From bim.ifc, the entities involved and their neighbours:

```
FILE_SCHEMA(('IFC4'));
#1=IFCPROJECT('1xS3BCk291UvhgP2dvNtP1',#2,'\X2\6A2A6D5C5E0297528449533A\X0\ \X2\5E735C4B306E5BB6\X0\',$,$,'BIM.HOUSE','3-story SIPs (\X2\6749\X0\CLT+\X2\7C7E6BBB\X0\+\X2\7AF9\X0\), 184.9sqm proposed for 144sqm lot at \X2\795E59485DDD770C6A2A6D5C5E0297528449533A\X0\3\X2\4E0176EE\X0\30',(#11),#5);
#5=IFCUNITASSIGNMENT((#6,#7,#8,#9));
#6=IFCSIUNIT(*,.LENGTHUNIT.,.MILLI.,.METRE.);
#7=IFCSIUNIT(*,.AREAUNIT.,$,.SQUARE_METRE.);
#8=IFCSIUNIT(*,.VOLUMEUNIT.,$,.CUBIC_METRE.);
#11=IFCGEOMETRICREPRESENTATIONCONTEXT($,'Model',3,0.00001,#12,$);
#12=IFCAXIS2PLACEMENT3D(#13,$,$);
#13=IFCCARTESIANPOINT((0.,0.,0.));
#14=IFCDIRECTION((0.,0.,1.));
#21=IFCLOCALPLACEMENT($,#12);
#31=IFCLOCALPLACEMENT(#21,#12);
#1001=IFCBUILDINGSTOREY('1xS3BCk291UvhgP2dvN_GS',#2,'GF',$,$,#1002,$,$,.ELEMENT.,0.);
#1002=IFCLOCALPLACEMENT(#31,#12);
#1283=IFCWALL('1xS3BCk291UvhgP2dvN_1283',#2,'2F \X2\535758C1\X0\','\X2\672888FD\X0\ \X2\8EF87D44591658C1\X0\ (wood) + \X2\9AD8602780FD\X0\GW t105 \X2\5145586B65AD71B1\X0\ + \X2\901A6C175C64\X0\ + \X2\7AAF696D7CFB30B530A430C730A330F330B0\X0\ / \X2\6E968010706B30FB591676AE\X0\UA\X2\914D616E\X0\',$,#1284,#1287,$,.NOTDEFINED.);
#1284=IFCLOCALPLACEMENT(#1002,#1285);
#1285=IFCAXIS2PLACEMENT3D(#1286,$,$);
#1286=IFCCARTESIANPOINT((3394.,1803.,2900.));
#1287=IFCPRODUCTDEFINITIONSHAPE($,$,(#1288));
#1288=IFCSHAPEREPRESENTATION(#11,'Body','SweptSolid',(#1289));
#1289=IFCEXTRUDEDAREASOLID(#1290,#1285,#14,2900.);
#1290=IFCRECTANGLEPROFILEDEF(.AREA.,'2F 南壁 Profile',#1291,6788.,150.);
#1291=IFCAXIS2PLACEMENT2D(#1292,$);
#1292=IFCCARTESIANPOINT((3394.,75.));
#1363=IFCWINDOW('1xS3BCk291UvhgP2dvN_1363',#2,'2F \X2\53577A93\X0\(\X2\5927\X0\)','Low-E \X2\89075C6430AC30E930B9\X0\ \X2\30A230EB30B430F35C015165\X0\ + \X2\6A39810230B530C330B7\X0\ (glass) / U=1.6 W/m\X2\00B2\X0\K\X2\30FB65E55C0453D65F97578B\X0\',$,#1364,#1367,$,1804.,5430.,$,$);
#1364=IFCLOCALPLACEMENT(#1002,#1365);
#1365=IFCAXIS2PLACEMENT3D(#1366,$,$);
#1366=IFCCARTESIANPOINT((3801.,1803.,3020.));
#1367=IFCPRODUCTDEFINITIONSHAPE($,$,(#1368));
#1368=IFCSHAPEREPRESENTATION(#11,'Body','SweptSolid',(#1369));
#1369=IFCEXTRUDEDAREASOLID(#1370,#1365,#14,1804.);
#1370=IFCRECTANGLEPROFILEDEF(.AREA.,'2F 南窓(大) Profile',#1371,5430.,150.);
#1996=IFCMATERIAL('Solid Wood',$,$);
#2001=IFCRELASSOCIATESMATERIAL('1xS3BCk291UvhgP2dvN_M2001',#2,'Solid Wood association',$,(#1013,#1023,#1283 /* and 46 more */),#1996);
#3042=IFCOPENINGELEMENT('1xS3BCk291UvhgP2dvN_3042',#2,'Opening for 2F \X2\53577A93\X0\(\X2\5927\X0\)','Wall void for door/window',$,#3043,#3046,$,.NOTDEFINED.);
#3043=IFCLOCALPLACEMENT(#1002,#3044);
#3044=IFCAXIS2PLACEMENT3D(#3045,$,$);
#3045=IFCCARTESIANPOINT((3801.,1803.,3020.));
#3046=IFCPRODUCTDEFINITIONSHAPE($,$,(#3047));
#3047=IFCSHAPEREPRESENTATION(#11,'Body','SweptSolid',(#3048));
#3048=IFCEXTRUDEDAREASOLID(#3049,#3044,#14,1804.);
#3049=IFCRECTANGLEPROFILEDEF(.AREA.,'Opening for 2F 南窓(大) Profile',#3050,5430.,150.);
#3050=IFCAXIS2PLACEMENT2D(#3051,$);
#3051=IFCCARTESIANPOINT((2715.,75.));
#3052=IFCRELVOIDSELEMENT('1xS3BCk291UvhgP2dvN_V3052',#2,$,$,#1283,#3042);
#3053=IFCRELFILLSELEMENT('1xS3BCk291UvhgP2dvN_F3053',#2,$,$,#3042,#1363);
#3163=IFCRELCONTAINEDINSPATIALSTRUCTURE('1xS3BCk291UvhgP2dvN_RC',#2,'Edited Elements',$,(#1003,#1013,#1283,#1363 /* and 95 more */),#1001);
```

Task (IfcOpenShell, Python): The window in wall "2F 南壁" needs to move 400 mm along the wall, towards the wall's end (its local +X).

```python
import ifcopenshell
import ifcopenshell.api.geometry
import ifcopenshell.util.placement
import ifcopenshell.util.unit

model = ifcopenshell.open("bim.ifc")
unit_scale = ifcopenshell.util.unit.calculate_unit_scale(model)

window = model.by_guid("1xS3BCk291UvhgP2dvN_1363")
opening = window.FillsVoids[0].RelatingOpeningElement
wall = opening.VoidsElements[0].RelatingBuildingElement

wall_matrix = ifcopenshell.util.placement.get_local_placement(wall.ObjectPlacement)
shift = wall_matrix[:3, 0] * 0.4 / unit_scale
before = ifcopenshell.util.placement.get_local_placement(window.ObjectPlacement)[:3, 3].copy()

# The window is not placed relative to its opening, so move both.
for product in (opening, window):
    matrix = ifcopenshell.util.placement.get_local_placement(product.ObjectPlacement)
    matrix[:3, 3] += shift
    ifcopenshell.api.geometry.edit_object_placement(model, product=product, matrix=matrix, is_si=False)

after = ifcopenshell.util.placement.get_local_placement(window.ObjectPlacement)[:3, 3]
print("window moved by", (after - before).round(3) + 0.0)

model.write("bim_v2.ifc")
```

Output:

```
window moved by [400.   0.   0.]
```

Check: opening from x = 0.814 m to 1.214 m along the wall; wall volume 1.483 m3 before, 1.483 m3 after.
